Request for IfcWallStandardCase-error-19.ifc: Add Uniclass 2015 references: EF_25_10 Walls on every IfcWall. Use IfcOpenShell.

First a look at what the model holds.

```python
import ifcopenshell

model = ifcopenshell.open("IfcWallStandardCase-error-19.ifc")
print(model.schema)
print("classifications:", [c.Name for c in model.by_type("IfcClassification")])
for ifc_class in ("IfcDoor", "IfcRoof", "IfcStair", "IfcWall", "IfcWindow"):
    print(ifc_class, len(model.by_type(ifc_class)))
```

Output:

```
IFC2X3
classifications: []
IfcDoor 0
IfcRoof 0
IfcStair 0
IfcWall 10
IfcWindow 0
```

```python
import ifcopenshell
import ifcopenshell.api.classification

model = ifcopenshell.open("IfcWallStandardCase-error-19.ifc")

# IFC2X3 requires Source and Edition and has no link from the project to the system.
system = model.create_entity("IfcClassification", Source="NBS", Edition="2015", Name="Uniclass 2015")

codes = {
    "IfcWall": ("EF_25_10", "Walls"),
}
for ifc_class, (code, name) in codes.items():
    products = model.by_type(ifc_class)
    ifcopenshell.api.classification.add_reference(
        model, products=products, classification=system, identification=code, name=name
    )
    print(code, len(products))

model.write("IfcWallStandardCase-error-19_v2.ifc")
```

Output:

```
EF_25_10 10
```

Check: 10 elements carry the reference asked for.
